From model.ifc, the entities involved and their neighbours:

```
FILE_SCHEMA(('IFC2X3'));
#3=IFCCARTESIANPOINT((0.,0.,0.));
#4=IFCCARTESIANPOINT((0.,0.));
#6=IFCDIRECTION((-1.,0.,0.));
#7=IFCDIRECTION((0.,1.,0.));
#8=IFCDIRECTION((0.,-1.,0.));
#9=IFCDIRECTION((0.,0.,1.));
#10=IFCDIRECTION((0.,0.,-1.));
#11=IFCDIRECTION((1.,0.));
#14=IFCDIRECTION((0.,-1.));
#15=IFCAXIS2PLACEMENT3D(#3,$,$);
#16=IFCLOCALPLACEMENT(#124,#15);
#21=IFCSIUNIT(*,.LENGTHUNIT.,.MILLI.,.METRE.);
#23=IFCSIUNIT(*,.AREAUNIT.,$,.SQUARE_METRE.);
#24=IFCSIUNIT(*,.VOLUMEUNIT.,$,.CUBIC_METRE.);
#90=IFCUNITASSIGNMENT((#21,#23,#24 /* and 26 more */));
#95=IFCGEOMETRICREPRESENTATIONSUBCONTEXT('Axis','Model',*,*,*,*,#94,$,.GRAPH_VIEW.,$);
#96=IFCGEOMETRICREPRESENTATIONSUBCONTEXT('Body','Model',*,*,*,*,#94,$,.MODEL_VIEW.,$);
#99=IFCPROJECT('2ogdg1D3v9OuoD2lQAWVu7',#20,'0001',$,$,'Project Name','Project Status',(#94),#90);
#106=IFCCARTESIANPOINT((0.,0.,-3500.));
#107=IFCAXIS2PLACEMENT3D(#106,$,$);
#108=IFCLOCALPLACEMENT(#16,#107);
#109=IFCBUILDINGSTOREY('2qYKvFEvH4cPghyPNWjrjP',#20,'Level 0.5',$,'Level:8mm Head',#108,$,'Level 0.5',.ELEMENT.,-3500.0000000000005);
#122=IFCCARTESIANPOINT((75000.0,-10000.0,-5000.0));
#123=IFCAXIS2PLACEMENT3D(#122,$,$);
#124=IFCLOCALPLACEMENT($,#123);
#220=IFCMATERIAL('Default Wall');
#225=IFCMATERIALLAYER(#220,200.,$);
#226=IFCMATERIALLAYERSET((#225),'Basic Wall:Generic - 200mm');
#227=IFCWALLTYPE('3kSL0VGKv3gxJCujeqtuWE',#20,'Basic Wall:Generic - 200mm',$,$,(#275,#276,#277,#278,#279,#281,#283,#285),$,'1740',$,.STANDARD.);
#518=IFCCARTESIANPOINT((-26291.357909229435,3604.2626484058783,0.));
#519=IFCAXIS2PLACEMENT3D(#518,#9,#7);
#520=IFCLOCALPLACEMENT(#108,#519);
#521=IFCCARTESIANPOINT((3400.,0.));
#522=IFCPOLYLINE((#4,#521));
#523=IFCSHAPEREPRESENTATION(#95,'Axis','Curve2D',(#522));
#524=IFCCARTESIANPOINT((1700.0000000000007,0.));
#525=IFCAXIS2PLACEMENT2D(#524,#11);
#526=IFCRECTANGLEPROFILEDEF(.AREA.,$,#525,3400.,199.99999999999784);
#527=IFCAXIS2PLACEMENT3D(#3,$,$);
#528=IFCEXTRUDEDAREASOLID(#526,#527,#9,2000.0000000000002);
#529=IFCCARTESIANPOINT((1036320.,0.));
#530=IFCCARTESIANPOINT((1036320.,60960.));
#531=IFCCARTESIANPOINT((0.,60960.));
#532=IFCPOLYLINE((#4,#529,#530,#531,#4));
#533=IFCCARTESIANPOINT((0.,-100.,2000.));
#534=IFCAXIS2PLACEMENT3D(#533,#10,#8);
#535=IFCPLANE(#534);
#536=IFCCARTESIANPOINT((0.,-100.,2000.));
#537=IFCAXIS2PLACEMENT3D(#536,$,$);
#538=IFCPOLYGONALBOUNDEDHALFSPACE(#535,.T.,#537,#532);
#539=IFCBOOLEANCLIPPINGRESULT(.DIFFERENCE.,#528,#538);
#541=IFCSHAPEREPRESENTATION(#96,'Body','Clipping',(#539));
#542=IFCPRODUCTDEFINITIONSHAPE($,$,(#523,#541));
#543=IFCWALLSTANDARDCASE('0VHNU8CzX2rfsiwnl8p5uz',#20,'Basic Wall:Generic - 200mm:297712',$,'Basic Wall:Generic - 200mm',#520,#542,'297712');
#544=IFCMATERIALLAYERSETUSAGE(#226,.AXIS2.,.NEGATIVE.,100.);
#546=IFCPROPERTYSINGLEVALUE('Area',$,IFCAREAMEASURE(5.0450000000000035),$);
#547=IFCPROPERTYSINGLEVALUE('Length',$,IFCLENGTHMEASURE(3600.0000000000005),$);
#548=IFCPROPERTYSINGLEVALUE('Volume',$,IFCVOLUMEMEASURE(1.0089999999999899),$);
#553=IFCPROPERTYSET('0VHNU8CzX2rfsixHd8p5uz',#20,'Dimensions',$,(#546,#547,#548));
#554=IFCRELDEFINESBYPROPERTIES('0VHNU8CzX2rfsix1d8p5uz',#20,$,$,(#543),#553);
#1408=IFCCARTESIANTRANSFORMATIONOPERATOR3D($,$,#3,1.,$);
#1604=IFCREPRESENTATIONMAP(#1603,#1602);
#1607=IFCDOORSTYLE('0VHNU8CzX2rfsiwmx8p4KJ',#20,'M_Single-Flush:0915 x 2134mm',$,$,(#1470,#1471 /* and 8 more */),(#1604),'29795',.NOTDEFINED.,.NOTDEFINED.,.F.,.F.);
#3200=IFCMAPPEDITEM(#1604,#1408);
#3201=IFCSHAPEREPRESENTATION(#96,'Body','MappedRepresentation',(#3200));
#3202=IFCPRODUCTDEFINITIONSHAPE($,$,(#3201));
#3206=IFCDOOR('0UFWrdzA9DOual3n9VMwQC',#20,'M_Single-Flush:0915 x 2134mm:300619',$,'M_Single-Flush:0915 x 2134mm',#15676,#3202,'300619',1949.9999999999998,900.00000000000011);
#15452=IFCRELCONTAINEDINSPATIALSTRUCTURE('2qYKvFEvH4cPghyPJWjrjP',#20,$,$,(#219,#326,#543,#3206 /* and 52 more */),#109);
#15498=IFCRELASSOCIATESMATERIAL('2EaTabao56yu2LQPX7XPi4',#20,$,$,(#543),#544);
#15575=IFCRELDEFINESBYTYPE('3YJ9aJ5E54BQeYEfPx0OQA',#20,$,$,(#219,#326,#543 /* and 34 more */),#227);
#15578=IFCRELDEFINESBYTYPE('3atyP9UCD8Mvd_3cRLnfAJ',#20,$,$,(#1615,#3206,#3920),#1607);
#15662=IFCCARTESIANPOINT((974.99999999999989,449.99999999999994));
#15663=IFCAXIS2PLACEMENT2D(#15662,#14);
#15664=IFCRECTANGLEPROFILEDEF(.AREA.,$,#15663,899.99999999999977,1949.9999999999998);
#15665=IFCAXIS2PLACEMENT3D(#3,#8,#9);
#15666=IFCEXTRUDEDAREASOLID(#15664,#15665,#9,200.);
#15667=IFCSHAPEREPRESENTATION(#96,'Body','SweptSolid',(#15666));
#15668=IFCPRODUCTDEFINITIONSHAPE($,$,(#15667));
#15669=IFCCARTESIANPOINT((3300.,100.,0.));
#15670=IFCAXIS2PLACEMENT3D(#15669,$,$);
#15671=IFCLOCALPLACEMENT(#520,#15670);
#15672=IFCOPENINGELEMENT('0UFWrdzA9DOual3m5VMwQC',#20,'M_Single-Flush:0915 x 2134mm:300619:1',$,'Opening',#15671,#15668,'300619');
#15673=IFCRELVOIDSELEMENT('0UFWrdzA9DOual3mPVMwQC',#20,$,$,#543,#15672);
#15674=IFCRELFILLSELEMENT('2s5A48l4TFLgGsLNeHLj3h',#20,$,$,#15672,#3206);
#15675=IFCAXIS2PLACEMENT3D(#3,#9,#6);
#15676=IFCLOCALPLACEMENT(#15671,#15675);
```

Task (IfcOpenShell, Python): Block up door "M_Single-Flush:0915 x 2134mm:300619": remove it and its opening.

```python
import ifcopenshell
import ifcopenshell.api.feature
import ifcopenshell.api.pset
import ifcopenshell.api.root
import ifcopenshell.geom
import ifcopenshell.util.element
import ifcopenshell.util.shape
import ifcopenshell.util.unit

model = ifcopenshell.open("model.ifc")
area_scale = ifcopenshell.util.unit.calculate_unit_scale(model, "AREAUNIT")
volume_scale = ifcopenshell.util.unit.calculate_unit_scale(model, "VOLUMEUNIT")
settings = ifcopenshell.geom.settings()


def volume(element):
    """Net volume in cubic metres, openings subtracted."""
    shape = ifcopenshell.geom.create_shape(settings, element)
    return ifcopenshell.util.shape.get_volume(shape.geometry)


door = model.by_id(3206)
opening = door.FillsVoids[0].RelatingOpeningElement
wall = opening.VoidsElements[0].RelatingBuildingElement
before = volume(wall)

ifcopenshell.api.root.remove_product(model, product=door)
ifcopenshell.api.feature.remove_feature(model, feature=opening)

after = volume(wall)
thickness = 0.2  # wall thickness in metres

# Update the wall's stored quantities.
pset = model.by_id(ifcopenshell.util.element.get_pset(wall, "Dimensions", should_inherit=False)["id"])
ifcopenshell.api.pset.edit_pset(model, pset=pset, properties={
    "Area": model.create_entity("IfcAreaMeasure", after / thickness / area_scale),
    "Volume": model.create_entity("IfcVolumeMeasure", after / volume_scale),
})

print(f"wall volume {before:.3f} -> {after:.3f} m3")

model.write("model_v2.ifc")
```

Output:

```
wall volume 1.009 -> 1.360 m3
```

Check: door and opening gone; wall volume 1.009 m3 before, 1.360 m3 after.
